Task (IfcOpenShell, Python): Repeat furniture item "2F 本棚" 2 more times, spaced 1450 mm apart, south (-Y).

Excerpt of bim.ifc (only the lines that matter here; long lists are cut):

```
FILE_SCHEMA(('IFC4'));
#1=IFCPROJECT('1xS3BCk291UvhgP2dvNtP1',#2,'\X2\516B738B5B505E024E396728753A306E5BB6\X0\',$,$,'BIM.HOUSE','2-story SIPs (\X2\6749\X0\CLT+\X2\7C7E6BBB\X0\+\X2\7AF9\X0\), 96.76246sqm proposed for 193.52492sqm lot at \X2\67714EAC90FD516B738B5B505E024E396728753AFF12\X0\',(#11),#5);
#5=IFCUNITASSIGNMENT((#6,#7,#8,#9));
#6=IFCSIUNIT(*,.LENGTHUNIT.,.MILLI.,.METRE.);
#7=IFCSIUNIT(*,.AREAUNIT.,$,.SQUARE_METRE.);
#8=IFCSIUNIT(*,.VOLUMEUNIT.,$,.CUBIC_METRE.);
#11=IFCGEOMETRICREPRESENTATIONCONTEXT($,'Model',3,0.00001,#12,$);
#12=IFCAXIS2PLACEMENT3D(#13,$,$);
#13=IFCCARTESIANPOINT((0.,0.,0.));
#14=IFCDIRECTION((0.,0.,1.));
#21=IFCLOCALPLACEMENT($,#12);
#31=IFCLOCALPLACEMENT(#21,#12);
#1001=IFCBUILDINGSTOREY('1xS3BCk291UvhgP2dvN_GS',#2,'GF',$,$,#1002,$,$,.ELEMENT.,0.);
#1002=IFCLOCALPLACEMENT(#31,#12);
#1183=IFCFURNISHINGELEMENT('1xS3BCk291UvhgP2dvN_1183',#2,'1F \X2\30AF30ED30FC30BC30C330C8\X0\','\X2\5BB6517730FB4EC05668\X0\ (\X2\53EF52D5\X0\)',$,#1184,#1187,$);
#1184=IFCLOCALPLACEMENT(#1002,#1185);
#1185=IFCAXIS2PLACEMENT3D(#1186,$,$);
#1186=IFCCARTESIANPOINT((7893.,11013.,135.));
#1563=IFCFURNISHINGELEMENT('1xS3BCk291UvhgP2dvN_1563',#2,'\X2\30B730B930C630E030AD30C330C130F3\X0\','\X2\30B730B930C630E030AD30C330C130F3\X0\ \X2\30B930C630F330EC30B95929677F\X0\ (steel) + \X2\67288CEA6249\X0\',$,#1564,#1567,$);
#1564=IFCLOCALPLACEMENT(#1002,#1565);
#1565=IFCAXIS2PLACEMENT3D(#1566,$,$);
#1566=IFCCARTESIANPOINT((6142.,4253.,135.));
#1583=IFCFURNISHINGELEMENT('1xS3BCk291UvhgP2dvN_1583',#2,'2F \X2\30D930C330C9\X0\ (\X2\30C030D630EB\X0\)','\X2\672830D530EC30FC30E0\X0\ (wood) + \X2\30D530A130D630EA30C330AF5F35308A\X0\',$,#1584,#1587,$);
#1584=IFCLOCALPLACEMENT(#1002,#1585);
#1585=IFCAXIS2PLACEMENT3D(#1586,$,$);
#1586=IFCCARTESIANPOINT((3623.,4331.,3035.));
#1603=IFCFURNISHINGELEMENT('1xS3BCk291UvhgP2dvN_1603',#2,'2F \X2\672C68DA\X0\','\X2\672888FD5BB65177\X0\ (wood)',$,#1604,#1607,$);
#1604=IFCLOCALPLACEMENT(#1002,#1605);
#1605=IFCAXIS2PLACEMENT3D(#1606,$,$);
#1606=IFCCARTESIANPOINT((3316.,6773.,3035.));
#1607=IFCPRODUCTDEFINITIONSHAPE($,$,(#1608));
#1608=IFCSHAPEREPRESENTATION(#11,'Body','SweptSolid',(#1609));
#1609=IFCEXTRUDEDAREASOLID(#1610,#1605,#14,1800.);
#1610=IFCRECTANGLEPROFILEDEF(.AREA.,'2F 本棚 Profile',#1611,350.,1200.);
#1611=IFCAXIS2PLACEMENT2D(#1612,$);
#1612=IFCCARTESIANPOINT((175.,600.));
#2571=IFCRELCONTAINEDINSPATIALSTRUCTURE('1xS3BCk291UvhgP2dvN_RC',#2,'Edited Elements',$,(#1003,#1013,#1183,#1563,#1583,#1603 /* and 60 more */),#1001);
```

```python
import numpy as np
import ifcopenshell
import ifcopenshell.api.geometry
import ifcopenshell.api.root
import ifcopenshell.util.element
import ifcopenshell.util.placement
import ifcopenshell.util.unit

model = ifcopenshell.open("bim.ifc")
unit_scale = ifcopenshell.util.unit.calculate_unit_scale(model)


def reuse_history(source, copy):
    """copy_class also copies each property set's owner history, people and application; keep the originals."""
    for rel in copy.IsDefinedBy:
        if rel.is_a("IfcRelDefinesByProperties") and (history := rel.RelatingPropertyDefinition.OwnerHistory):
            rel.RelatingPropertyDefinition.OwnerHistory = source.OwnerHistory
            ifcopenshell.util.element.remove_deep2(model, history)


source = model.by_guid("1xS3BCk291UvhgP2dvN_1603")
base = ifcopenshell.util.placement.get_local_placement(source.ObjectPlacement)
step = np.array([0.0, -1.0, 0.0]) * 1.45 / unit_scale

for i in range(1, 3):
    copy = ifcopenshell.api.root.copy_class(model, product=source)
    copy.Representation = ifcopenshell.util.element.copy_deep(
        model, source.Representation, exclude=["IfcGeometricRepresentationContext", "IfcRepresentationMap"]
    )
    reuse_history(source, copy)
    matrix = base.copy()
    matrix[:3, 3] += i * step
    print("added at", matrix[:3, 3].round(3) + 0.0)
    ifcopenshell.api.geometry.edit_object_placement(model, product=copy, matrix=matrix, is_si=False)

model.write("bim_v2.ifc")
```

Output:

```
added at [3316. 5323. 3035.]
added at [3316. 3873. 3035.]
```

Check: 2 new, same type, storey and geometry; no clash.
